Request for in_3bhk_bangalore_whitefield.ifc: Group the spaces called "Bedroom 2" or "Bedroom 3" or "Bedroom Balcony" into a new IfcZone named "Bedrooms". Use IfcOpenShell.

First a look at what the model holds.

```python
import ifcopenshell

model = ifcopenshell.open("in_3bhk_bangalore_whitefield.ifc")
print(model.schema)
seen = {}
for space in model.by_type("IfcSpace"):
    seen[space.LongName] = seen.get(space.LongName, 0) + 1
for name, count in sorted(seen.items(), key=str):
    print(count, "x", name)
print("zones:", [z.Name for z in model.by_type("IfcZone")][:20])
```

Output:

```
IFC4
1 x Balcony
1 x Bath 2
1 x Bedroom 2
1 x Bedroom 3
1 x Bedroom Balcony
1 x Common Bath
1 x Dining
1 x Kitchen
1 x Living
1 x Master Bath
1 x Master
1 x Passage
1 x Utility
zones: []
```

```python
import ifcopenshell
import ifcopenshell.api.group
import ifcopenshell.api.root

model = ifcopenshell.open("in_3bhk_bangalore_whitefield.ifc")

names = {"Bedroom 2", "Bedroom 3", "Bedroom Balcony"}
spaces = [s for s in model.by_type("IfcSpace") if s.LongName in names]

zone = ifcopenshell.api.root.create_entity(model, ifc_class="IfcZone", name="Bedrooms")
ifcopenshell.api.group.assign_group(model, products=spaces, group=zone)
print(len(spaces), "spaces in", zone.Name)

model.write("in_3bhk_bangalore_whitefield_updated.ifc")
```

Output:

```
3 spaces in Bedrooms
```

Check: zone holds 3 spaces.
